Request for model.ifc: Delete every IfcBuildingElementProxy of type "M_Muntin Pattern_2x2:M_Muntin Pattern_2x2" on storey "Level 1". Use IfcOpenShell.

First a look at what the model holds.

```python
import ifcopenshell
import ifcopenshell.util.element

model = ifcopenshell.open("model.ifc")
print(model.schema)
storey = next(s for s in model.by_type("IfcBuildingStorey") if s.Name == "Level 1")
proxies = [e for e in ifcopenshell.util.element.get_decomposition(storey) if e.is_a("IfcBuildingElementProxy")]
seen = {}
for e in proxies:
    element_type = ifcopenshell.util.element.get_type(e)
    name = element_type.Name if element_type not in (None, e) else None
    seen[name] = seen.get(name, 0) + 1
for name, count in sorted(seen.items(), key=str):
    print(count, "x", name)
```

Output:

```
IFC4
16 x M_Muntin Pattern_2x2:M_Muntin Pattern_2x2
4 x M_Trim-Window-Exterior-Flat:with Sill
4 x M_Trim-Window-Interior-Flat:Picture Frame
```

```python
import ifcopenshell
import ifcopenshell.api.root
import ifcopenshell.util.element

model = ifcopenshell.open("model.ifc")

storey = next(s for s in model.by_type("IfcBuildingStorey") if s.Name == "Level 1")
proxies = [e for e in ifcopenshell.util.element.get_decomposition(storey) if e.is_a("IfcBuildingElementProxy")]
targets = [e for e in proxies if (t := ifcopenshell.util.element.get_type(e)) not in (None, e) and t.Name == "M_Muntin Pattern_2x2:M_Muntin Pattern_2x2"]

for e in targets:
    ifcopenshell.api.root.remove_product(model, product=e)
print(len(targets), "removed")

model.write("model-out.ifc")
```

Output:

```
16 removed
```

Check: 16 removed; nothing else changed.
